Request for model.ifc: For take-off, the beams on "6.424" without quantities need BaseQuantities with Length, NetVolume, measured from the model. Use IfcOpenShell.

First a look at what the model holds.

```python
import ifcopenshell
import ifcopenshell.util.element
import ifcopenshell.util.unit

model = ifcopenshell.open("model.ifc")
print(model.schema)
for unit_type in ("LENGTHUNIT", "AREAUNIT", "VOLUMEUNIT"):
    print(unit_type, ifcopenshell.util.unit.calculate_unit_scale(model, unit_type))
storey = next(s for s in model.by_type("IfcBuildingStorey") if s.Name == "6.424")
beams = [e for e in ifcopenshell.util.element.get_decomposition(storey) if e.is_a("IfcBeam")]
for e in sorted(beams, key=lambda e: e.id()):
    print(e.id(), e.is_a(), e.Name, list(ifcopenshell.util.element.get_psets(e, qtos_only=True)), sep=" | ")
```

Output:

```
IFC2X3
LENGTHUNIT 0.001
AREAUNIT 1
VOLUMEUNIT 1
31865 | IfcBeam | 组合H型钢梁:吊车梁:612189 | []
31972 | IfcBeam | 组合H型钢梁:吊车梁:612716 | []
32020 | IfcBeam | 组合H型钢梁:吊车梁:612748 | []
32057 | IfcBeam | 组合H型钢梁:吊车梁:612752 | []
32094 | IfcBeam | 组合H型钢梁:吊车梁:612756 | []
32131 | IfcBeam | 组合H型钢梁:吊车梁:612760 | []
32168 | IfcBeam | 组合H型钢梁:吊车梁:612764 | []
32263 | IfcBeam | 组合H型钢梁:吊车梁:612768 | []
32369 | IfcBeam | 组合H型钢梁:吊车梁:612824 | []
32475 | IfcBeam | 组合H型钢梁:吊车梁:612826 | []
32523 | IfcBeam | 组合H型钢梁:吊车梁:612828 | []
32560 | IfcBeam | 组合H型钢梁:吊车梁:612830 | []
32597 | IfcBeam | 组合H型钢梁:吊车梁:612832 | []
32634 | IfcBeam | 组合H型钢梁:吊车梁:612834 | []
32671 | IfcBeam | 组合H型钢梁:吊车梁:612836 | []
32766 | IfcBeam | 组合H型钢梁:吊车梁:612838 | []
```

```python
import ifcopenshell
import ifcopenshell.api.pset
import ifcopenshell.geom
import ifcopenshell.util.element
import ifcopenshell.util.shape
import ifcopenshell.util.unit

model = ifcopenshell.open("model.ifc")
unit_scale = ifcopenshell.util.unit.calculate_unit_scale(model)
volume_scale = ifcopenshell.util.unit.calculate_unit_scale(model, "VOLUMEUNIT")
settings = ifcopenshell.geom.settings()

storey = next(s for s in model.by_type("IfcBuildingStorey") if s.Name == "6.424")
beams = [e for e in ifcopenshell.util.element.get_decomposition(storey) if e.is_a("IfcBeam")]

for e in sorted(beams, key=lambda e: e.id()):
    if ifcopenshell.util.element.get_psets(e, qtos_only=True, should_inherit=False):
        continue
    # Geometry comes back in metres, in the element's own axes.
    shape = ifcopenshell.geom.create_shape(settings, e)
    values = {
        "Length": ifcopenshell.util.shape.get_max_xyz(shape.geometry) / unit_scale,
        "NetVolume": ifcopenshell.util.shape.get_volume(shape.geometry) / volume_scale,
    }
    qto = ifcopenshell.api.pset.add_qto(model, product=e, name="BaseQuantities")
    ifcopenshell.api.pset.edit_qto(model, qto=qto, properties=values)
    print(e.id(), {k: round(v, 3) for k, v in values.items()})

model.write("model_rev.ifc")
```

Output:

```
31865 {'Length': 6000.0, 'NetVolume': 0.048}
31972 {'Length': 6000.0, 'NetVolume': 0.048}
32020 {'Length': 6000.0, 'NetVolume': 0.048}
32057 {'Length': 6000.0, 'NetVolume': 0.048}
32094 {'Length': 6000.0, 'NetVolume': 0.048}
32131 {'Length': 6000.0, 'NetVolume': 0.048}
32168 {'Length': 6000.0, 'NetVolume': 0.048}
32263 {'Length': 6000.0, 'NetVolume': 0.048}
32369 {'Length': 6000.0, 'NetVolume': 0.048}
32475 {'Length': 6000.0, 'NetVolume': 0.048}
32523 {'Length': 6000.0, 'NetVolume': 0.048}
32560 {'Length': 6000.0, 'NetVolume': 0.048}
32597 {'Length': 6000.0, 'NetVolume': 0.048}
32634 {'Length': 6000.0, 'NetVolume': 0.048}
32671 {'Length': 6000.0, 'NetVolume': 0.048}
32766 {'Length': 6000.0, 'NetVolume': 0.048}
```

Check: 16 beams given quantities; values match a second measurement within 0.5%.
